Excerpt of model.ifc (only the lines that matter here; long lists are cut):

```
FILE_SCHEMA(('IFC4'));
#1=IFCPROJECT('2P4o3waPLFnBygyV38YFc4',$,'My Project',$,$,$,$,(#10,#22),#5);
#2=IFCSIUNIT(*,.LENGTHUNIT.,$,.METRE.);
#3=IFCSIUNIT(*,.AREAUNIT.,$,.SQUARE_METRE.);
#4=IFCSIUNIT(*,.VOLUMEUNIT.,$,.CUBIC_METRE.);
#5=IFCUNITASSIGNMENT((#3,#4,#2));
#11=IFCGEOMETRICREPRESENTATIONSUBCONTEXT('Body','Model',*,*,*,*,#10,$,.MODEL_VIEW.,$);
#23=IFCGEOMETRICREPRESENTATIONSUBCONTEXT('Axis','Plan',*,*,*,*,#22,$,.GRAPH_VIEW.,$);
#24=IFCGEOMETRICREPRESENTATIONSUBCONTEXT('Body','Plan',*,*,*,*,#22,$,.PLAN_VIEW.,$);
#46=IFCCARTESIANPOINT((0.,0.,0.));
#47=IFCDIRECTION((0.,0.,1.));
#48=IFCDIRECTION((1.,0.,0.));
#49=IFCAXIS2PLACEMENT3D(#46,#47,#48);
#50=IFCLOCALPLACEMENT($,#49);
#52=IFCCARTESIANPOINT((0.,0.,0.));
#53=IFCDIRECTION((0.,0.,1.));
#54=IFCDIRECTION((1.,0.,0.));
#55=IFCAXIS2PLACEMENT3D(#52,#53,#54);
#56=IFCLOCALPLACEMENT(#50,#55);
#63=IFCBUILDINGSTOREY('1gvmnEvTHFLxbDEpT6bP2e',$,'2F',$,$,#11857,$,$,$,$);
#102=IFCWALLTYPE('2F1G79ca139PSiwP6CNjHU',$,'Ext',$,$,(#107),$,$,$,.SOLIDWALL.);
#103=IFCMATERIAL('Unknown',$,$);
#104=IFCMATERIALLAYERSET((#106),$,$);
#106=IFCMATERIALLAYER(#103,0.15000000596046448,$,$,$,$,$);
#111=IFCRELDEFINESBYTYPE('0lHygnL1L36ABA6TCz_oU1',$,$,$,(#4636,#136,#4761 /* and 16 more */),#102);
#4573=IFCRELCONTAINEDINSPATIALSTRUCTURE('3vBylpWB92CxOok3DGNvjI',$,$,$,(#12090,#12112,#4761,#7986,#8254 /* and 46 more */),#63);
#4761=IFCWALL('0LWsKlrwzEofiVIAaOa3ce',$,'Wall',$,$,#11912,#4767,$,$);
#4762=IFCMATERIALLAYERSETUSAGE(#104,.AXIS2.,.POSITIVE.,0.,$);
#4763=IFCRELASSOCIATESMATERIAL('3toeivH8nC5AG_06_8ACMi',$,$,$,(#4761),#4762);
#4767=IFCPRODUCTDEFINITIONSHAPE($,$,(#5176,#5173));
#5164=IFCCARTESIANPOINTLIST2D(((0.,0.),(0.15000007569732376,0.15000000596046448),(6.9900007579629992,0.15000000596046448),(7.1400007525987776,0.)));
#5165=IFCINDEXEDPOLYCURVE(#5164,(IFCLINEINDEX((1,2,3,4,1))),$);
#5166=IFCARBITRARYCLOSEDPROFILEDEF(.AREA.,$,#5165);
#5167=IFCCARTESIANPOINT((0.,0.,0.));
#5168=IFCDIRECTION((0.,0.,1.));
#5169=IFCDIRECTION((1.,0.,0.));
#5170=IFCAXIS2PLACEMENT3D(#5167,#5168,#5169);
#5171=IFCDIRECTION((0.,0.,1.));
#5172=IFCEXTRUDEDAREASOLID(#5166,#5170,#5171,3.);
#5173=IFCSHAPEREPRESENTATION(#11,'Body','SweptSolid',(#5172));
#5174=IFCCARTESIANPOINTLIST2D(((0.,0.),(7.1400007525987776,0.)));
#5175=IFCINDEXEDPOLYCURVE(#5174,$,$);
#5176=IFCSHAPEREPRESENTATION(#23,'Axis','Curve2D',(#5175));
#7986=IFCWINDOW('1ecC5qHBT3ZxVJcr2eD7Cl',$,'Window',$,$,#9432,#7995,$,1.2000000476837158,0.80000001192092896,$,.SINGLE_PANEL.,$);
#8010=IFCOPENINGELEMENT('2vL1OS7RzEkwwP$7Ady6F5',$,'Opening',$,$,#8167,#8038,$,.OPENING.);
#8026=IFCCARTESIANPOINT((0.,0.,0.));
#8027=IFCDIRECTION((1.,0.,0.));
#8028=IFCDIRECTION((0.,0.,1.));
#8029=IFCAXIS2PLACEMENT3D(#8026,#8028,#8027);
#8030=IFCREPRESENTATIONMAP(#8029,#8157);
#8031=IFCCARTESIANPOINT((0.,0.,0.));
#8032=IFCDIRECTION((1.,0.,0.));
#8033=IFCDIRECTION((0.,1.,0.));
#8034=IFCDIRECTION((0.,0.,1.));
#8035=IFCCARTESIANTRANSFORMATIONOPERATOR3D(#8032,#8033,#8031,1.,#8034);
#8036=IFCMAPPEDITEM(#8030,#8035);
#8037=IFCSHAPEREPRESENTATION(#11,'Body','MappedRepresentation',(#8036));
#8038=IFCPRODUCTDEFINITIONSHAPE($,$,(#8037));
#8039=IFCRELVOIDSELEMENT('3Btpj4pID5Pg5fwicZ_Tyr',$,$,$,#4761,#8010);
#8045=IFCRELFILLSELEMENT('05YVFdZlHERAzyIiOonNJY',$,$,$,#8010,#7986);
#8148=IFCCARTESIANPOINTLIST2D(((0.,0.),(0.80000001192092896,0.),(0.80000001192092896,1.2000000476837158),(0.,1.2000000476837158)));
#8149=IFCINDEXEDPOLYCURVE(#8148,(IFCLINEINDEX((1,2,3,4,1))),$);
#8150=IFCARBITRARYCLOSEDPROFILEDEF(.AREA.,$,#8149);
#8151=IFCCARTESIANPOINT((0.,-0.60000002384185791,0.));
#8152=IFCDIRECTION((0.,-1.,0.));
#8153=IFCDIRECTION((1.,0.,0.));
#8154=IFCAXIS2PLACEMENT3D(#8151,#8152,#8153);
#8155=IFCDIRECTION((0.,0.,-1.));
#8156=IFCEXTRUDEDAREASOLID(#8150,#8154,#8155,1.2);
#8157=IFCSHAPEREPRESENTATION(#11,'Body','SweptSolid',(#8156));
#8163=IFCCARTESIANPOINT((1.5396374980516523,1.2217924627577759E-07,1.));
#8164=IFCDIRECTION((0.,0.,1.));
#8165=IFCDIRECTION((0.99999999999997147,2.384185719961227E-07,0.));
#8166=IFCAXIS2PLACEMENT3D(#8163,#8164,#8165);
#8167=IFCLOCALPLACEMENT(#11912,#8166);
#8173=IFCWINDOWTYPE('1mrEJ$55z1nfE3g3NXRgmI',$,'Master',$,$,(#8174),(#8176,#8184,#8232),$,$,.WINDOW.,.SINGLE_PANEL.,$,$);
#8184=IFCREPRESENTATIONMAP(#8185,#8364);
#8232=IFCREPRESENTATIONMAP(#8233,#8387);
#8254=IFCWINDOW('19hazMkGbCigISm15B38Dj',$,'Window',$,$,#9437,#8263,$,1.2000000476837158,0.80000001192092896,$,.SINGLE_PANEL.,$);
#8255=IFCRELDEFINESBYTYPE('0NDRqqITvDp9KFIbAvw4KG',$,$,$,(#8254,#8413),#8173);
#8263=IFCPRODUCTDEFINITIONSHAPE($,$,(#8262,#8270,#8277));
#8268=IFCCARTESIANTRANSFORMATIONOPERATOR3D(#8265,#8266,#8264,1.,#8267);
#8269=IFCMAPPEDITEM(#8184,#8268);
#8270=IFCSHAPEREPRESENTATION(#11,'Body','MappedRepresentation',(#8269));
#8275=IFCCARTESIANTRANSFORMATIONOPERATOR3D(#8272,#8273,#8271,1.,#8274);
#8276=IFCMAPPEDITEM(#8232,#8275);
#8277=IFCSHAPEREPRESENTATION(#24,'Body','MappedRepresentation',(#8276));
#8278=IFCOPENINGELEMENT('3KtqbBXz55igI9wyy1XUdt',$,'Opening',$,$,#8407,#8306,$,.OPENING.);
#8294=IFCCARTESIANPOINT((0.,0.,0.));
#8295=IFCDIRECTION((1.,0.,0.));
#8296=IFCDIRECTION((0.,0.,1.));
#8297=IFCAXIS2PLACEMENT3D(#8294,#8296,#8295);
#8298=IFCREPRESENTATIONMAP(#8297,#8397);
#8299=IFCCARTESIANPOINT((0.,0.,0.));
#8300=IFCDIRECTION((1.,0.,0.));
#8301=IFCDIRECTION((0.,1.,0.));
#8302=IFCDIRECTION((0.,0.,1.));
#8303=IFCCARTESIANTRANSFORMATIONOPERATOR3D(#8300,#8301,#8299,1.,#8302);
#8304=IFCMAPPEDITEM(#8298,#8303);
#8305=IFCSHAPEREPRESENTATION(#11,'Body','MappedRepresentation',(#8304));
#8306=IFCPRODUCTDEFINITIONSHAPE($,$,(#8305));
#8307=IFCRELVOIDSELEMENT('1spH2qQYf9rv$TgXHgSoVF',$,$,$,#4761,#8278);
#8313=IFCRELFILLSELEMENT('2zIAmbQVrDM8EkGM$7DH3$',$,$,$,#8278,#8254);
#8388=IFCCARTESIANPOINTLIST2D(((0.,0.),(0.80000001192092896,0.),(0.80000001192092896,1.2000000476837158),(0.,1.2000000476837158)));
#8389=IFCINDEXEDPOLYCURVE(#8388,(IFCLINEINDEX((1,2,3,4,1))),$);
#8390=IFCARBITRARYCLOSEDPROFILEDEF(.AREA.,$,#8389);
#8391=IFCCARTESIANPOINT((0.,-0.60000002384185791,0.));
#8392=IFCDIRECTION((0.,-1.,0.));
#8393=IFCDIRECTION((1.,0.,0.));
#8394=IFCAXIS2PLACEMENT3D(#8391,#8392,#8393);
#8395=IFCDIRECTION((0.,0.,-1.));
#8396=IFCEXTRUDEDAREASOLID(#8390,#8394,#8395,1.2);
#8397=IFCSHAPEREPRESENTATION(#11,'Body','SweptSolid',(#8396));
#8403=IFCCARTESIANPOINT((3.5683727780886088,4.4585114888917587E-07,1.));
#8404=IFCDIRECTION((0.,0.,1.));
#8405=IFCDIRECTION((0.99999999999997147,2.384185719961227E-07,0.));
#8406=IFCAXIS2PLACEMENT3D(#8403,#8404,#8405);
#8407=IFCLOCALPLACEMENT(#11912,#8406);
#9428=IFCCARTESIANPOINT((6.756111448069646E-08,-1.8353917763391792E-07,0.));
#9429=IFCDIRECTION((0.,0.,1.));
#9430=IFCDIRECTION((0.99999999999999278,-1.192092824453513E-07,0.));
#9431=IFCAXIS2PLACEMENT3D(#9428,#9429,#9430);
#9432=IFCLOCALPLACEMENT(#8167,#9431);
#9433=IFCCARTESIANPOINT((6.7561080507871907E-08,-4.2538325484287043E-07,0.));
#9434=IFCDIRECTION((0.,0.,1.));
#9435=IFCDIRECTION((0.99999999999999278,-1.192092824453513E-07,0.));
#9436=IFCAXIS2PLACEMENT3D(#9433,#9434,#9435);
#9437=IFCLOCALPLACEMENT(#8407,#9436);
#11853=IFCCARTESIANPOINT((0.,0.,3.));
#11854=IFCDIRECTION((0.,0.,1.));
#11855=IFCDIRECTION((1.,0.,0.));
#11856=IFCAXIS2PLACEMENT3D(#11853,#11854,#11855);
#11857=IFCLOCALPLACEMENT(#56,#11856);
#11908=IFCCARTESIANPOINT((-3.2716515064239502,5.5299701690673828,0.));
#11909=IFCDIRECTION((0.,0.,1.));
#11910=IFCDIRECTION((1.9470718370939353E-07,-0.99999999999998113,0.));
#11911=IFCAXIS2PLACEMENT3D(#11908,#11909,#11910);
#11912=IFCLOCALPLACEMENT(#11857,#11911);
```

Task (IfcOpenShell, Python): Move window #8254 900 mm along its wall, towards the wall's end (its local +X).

```python
import ifcopenshell
import ifcopenshell.api.geometry
import ifcopenshell.util.placement

model = ifcopenshell.open("model.ifc")

window = model.by_guid("19hazMkGbCigISm15B38Dj")
opening = window.FillsVoids[0].RelatingOpeningElement
wall = opening.VoidsElements[0].RelatingBuildingElement

wall_matrix = ifcopenshell.util.placement.get_local_placement(wall.ObjectPlacement)
shift = wall_matrix[:3, 0] * 0.9
before = ifcopenshell.util.placement.get_local_placement(window.ObjectPlacement)[:3, 3].copy()

# The window is placed relative to its opening, so it follows when the opening moves.
matrix = ifcopenshell.util.placement.get_local_placement(opening.ObjectPlacement)
matrix[:3, 3] += shift
ifcopenshell.api.geometry.edit_object_placement(
    model, product=opening, matrix=matrix, is_si=False, should_transform_children=True
)

after = ifcopenshell.util.placement.get_local_placement(window.ObjectPlacement)[:3, 3]
print("window moved by", (after - before).round(3) + 0.0)

model.write("model_rev.ifc")
```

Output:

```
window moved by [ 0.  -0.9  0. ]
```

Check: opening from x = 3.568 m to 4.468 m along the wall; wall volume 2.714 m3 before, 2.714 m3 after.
